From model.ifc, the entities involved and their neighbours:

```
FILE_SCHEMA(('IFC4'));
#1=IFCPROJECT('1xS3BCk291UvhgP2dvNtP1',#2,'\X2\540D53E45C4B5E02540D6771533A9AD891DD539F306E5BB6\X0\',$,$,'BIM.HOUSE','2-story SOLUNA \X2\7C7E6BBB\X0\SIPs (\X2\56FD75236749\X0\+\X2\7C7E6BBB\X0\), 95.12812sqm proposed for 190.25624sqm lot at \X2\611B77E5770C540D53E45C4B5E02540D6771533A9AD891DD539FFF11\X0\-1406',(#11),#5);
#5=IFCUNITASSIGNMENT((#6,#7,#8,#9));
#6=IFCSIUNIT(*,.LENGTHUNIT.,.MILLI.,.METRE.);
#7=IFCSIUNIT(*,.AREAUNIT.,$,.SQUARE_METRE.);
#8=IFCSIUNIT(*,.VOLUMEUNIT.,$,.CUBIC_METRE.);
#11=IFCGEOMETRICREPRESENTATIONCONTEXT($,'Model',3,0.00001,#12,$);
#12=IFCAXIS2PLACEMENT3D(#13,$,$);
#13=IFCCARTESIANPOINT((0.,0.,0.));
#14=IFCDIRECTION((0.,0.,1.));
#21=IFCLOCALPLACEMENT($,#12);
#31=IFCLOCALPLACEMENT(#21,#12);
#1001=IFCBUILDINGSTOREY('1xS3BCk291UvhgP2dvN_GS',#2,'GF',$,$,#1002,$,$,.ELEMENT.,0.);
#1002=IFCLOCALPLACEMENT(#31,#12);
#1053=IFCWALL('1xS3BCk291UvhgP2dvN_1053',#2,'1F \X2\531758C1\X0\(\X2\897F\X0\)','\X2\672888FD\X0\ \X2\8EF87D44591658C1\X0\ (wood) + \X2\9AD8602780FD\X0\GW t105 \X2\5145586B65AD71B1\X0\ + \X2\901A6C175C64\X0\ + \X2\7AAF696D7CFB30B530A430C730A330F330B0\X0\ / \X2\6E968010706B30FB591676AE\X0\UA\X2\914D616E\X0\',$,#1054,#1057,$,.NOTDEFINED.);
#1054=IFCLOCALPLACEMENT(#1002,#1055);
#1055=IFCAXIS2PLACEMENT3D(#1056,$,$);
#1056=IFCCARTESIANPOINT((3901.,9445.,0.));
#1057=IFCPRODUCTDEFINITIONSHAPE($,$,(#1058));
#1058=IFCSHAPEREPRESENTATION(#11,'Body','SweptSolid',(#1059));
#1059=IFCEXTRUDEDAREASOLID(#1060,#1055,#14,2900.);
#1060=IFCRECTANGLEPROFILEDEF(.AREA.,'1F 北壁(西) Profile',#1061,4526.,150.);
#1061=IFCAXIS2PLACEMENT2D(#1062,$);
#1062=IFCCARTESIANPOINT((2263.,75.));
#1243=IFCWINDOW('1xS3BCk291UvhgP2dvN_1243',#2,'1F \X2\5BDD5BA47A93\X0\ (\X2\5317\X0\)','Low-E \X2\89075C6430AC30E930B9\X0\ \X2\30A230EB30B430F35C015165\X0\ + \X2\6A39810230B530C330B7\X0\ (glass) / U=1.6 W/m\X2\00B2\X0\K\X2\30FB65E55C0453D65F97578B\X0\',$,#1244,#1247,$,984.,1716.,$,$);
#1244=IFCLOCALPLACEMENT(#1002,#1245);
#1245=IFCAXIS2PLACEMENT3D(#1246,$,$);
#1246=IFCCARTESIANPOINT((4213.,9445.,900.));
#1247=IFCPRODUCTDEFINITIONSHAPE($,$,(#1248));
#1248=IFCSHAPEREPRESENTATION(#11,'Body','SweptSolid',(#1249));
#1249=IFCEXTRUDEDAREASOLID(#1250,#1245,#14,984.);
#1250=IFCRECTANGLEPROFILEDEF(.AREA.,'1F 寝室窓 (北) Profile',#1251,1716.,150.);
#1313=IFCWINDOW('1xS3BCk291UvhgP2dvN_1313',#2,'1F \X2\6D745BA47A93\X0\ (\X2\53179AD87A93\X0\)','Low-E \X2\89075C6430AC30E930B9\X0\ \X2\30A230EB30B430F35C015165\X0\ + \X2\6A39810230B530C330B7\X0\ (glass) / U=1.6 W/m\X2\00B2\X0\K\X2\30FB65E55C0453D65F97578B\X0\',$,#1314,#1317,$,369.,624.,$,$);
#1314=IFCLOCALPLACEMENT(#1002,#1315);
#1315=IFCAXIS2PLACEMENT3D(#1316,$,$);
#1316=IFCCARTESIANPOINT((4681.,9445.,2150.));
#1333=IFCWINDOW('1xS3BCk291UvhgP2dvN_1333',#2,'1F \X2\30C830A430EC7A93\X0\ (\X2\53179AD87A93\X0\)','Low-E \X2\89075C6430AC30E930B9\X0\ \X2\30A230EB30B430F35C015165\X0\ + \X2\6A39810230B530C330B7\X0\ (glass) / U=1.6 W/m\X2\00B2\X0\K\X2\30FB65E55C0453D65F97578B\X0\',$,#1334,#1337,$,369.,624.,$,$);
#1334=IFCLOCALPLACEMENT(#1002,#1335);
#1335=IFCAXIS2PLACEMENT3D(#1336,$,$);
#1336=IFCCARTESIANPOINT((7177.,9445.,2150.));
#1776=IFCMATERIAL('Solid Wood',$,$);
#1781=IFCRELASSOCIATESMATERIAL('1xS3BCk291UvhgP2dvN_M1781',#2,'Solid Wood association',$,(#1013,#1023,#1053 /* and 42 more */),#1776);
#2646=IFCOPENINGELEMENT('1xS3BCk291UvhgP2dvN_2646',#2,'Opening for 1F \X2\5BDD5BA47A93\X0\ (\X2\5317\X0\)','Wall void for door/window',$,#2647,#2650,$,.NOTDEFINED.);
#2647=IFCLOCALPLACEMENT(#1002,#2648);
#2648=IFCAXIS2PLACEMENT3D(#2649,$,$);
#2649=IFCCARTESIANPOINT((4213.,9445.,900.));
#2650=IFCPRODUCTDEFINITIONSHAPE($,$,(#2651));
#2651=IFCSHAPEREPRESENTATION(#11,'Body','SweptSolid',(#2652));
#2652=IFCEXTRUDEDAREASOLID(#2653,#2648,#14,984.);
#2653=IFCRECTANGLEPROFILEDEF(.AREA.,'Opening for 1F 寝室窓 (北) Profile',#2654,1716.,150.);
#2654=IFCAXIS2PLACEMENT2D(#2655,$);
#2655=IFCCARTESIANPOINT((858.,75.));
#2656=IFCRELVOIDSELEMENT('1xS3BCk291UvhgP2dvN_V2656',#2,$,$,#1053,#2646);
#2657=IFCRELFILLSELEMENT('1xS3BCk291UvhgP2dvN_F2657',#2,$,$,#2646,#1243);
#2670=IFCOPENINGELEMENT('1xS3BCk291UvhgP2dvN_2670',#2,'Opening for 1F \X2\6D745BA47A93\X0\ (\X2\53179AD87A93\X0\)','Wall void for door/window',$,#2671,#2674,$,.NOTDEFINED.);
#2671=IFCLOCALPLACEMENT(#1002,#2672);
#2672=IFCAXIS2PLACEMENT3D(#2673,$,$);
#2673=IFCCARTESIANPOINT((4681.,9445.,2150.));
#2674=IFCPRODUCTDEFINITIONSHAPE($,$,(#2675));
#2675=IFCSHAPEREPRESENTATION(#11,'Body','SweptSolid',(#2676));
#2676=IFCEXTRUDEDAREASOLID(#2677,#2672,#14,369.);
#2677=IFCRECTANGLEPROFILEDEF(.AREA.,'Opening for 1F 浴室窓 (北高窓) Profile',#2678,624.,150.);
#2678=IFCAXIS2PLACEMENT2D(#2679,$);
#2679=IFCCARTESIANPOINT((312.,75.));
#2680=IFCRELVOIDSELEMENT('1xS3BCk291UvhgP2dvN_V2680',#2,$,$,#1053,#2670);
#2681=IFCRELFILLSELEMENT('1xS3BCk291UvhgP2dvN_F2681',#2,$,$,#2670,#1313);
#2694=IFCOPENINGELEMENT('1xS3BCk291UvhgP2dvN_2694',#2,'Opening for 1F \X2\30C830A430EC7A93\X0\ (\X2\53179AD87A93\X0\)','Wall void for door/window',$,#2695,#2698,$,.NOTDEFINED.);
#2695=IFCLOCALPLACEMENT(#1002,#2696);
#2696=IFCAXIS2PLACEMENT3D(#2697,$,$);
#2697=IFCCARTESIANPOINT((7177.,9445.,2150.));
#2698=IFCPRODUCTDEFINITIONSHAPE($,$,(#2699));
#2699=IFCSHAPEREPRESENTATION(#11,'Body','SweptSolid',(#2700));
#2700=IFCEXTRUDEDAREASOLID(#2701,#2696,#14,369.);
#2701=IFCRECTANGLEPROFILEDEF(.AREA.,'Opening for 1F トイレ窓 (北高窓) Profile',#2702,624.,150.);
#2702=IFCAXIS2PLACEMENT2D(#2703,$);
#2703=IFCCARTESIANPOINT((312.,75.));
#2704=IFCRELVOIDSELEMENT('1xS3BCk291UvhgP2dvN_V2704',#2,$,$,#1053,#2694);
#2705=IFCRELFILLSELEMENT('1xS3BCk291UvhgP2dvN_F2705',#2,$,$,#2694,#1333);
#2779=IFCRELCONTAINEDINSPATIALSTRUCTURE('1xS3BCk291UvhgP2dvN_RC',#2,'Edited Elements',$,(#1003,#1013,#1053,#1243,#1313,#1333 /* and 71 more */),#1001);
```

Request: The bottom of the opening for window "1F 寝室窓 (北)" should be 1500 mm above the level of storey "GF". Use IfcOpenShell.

```python
import numpy as np
import ifcopenshell
import ifcopenshell.api.geometry
import ifcopenshell.geom
import ifcopenshell.util.element
import ifcopenshell.util.placement
import ifcopenshell.util.shape
import ifcopenshell.util.unit

model = ifcopenshell.open("model.ifc")
unit_scale = ifcopenshell.util.unit.calculate_unit_scale(model)

window = model.by_id(1243)
opening = window.FillsVoids[0].RelatingOpeningElement
storey = ifcopenshell.util.element.get_container(window, ifc_class="IfcBuildingStorey")
level = ifcopenshell.util.placement.get_local_placement(storey.ObjectPlacement)[2, 3]

# The opening's origin need not be at the sill, so measure its lowest point.
shape = ifcopenshell.geom.create_shape(ifcopenshell.geom.settings(), opening)
bottom = ifcopenshell.util.shape.get_shape_bottom_elevation(shape, shape.geometry) / unit_scale
dz = level + 1500.0 - bottom

shift = np.array([0.0, 0.0, dz])
# The window is not placed relative to its opening, so move both.
for product in (opening, window):
    matrix = ifcopenshell.util.placement.get_local_placement(product.ObjectPlacement)
    matrix[:3, 3] += shift
    ifcopenshell.api.geometry.edit_object_placement(model, product=product, matrix=matrix, is_si=False)

print(f"moved by {dz * unit_scale:+.3f} m")

model.write("model_edited.ifc")
```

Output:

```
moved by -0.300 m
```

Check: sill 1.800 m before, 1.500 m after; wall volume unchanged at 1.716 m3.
